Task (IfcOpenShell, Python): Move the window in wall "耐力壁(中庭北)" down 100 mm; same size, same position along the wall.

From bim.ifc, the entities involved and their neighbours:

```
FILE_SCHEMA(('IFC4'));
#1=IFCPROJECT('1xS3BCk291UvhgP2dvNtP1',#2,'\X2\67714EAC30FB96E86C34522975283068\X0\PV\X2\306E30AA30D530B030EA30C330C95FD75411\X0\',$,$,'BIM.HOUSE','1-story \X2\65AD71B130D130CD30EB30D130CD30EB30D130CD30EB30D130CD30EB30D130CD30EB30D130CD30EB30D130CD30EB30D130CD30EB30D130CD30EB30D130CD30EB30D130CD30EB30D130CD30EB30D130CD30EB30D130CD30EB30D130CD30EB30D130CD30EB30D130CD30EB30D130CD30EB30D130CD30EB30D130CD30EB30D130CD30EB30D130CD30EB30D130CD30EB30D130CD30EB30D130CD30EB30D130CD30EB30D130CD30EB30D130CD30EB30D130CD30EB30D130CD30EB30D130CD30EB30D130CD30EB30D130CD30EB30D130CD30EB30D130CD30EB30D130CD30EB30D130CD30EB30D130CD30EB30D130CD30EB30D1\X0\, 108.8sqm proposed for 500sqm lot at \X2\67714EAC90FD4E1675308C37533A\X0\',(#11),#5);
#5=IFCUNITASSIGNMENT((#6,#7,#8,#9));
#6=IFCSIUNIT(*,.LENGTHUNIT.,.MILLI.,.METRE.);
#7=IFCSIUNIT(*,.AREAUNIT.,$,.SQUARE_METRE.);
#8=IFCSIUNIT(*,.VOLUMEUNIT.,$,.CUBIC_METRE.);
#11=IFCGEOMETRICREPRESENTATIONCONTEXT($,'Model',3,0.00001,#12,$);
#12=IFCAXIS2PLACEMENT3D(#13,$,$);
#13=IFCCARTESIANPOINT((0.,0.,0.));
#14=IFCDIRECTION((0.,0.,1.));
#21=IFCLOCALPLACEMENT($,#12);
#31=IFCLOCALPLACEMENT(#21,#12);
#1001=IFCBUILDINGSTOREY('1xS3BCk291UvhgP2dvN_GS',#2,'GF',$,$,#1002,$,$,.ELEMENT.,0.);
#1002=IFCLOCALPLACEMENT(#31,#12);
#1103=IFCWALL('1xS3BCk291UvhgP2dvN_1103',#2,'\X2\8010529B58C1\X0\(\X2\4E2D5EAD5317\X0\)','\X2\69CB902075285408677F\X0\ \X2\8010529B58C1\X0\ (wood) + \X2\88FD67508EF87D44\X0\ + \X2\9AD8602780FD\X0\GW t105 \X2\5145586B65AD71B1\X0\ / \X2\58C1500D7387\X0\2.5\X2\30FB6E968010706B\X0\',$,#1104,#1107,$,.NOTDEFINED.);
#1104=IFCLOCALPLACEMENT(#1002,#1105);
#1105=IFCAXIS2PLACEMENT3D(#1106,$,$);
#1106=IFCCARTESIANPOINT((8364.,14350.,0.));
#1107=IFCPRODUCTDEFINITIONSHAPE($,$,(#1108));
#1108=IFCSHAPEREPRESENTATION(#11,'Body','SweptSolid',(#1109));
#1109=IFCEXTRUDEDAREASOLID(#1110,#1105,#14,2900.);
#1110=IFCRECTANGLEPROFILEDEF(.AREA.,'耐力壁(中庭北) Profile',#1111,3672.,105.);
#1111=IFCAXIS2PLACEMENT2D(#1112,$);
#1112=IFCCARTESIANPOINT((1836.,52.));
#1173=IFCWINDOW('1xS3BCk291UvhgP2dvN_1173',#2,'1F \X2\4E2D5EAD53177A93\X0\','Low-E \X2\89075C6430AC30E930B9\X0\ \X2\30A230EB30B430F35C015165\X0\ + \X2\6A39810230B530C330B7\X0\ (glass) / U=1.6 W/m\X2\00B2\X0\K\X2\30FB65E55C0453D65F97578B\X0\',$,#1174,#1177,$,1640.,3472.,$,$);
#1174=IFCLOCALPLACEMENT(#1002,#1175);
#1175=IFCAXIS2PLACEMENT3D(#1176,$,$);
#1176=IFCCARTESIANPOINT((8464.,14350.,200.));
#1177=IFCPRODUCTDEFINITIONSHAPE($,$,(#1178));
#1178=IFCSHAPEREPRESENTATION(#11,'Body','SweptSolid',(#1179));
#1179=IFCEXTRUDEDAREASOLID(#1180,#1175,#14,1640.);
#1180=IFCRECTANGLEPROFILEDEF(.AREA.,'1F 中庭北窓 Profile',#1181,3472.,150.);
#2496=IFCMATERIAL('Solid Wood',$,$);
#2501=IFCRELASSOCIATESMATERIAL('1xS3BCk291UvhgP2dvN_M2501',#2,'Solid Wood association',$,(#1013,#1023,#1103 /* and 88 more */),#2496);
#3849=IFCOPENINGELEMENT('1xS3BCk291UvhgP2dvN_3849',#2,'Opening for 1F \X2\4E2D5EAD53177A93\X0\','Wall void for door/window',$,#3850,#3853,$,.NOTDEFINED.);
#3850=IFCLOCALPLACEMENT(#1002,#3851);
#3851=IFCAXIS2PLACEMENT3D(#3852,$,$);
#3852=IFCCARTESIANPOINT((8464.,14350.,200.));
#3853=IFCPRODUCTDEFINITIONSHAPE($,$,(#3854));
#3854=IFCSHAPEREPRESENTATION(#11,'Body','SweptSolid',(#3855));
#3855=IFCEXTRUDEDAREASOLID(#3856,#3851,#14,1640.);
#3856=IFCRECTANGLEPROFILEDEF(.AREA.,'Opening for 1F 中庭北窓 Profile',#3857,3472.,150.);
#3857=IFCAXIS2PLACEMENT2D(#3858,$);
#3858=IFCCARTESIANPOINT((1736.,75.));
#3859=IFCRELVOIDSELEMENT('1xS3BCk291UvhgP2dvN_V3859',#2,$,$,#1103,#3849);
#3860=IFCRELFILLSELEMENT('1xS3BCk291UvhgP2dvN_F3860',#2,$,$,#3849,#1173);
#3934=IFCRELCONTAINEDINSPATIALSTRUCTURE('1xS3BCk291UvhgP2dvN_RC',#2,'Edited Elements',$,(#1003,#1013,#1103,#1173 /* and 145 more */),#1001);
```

```python
import numpy as np
import ifcopenshell
import ifcopenshell.api.geometry
import ifcopenshell.util.placement
import ifcopenshell.util.unit

model = ifcopenshell.open("bim.ifc")
unit_scale = ifcopenshell.util.unit.calculate_unit_scale(model)

window = model.by_guid("1xS3BCk291UvhgP2dvN_1173")
opening = window.FillsVoids[0].RelatingOpeningElement
dz = -0.1 / unit_scale

shift = np.array([0.0, 0.0, dz])
# The window is not placed relative to its opening, so move both.
for product in (opening, window):
    matrix = ifcopenshell.util.placement.get_local_placement(product.ObjectPlacement)
    matrix[:3, 3] += shift
    ifcopenshell.api.geometry.edit_object_placement(model, product=product, matrix=matrix, is_si=False)

print(f"moved by {dz * unit_scale:+.3f} m")

model.write("bim_v2.ifc")
```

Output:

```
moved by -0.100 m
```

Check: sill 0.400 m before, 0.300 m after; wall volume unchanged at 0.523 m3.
